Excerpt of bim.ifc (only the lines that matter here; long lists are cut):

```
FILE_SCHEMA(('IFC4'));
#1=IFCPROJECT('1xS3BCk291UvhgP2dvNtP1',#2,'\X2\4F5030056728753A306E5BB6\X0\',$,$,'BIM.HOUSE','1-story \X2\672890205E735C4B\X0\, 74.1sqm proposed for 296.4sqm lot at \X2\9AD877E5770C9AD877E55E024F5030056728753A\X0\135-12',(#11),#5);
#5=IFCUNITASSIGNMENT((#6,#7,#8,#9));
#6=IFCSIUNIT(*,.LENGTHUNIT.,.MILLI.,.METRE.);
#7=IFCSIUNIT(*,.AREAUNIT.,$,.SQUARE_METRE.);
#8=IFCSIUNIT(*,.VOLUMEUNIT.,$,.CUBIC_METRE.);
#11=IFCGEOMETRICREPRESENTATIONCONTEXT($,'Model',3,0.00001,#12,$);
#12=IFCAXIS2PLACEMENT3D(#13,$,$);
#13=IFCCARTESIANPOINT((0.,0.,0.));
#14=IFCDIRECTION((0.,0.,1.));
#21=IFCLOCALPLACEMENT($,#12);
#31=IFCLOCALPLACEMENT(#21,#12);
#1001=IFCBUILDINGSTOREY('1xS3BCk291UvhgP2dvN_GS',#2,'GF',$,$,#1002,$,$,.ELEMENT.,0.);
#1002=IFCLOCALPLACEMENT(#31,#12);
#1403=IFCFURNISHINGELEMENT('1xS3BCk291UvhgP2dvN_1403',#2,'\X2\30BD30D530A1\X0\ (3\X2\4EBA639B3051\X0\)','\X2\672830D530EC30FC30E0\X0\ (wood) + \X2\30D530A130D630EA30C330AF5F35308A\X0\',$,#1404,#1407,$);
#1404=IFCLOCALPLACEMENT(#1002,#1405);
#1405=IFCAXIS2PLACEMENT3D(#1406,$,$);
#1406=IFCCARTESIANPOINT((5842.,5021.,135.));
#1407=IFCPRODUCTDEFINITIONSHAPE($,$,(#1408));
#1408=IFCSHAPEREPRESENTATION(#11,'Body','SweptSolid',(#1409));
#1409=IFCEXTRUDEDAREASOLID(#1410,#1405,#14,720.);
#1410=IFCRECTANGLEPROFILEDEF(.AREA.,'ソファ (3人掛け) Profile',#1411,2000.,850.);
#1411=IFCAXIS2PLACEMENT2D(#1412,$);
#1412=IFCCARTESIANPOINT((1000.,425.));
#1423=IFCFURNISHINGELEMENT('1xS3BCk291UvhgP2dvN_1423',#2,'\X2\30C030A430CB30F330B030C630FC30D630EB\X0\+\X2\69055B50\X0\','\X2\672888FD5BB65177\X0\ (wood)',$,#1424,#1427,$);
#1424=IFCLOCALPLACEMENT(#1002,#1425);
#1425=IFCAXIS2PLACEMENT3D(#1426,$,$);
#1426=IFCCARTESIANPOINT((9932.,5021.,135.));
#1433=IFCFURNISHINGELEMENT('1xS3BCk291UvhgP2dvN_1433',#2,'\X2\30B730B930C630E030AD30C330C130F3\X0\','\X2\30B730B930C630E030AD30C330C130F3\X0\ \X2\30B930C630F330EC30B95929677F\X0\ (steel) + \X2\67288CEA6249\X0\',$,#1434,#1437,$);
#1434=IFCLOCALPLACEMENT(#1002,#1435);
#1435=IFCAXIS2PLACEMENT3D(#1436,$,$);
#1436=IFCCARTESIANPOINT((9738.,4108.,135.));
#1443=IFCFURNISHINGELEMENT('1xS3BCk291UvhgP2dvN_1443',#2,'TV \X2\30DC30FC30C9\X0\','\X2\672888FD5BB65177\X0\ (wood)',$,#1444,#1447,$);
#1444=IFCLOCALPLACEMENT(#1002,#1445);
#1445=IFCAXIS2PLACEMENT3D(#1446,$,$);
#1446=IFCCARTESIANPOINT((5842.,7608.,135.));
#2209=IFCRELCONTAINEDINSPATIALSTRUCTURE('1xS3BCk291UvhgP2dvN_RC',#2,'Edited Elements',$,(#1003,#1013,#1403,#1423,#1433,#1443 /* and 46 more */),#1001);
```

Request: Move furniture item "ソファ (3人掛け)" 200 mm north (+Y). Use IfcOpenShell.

```python
import ifcopenshell
import ifcopenshell.api.geometry
import ifcopenshell.util.placement
import ifcopenshell.util.unit

model = ifcopenshell.open("bim.ifc")
unit_scale = ifcopenshell.util.unit.calculate_unit_scale(model)

item = model.by_guid("1xS3BCk291UvhgP2dvN_1403")
matrix = ifcopenshell.util.placement.get_local_placement(item.ObjectPlacement)
matrix[1, 3] += 0.2 / unit_scale
ifcopenshell.api.geometry.edit_object_placement(model, product=item, matrix=matrix, is_si=False)

print(ifcopenshell.util.placement.get_local_placement(item.ObjectPlacement).round(3) + 0.0)

model.write("bim_v2.ifc")
```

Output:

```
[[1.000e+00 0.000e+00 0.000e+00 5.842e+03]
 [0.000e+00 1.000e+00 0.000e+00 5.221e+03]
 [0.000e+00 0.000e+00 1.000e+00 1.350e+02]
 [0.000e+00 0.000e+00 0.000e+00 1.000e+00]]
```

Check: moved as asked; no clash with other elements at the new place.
